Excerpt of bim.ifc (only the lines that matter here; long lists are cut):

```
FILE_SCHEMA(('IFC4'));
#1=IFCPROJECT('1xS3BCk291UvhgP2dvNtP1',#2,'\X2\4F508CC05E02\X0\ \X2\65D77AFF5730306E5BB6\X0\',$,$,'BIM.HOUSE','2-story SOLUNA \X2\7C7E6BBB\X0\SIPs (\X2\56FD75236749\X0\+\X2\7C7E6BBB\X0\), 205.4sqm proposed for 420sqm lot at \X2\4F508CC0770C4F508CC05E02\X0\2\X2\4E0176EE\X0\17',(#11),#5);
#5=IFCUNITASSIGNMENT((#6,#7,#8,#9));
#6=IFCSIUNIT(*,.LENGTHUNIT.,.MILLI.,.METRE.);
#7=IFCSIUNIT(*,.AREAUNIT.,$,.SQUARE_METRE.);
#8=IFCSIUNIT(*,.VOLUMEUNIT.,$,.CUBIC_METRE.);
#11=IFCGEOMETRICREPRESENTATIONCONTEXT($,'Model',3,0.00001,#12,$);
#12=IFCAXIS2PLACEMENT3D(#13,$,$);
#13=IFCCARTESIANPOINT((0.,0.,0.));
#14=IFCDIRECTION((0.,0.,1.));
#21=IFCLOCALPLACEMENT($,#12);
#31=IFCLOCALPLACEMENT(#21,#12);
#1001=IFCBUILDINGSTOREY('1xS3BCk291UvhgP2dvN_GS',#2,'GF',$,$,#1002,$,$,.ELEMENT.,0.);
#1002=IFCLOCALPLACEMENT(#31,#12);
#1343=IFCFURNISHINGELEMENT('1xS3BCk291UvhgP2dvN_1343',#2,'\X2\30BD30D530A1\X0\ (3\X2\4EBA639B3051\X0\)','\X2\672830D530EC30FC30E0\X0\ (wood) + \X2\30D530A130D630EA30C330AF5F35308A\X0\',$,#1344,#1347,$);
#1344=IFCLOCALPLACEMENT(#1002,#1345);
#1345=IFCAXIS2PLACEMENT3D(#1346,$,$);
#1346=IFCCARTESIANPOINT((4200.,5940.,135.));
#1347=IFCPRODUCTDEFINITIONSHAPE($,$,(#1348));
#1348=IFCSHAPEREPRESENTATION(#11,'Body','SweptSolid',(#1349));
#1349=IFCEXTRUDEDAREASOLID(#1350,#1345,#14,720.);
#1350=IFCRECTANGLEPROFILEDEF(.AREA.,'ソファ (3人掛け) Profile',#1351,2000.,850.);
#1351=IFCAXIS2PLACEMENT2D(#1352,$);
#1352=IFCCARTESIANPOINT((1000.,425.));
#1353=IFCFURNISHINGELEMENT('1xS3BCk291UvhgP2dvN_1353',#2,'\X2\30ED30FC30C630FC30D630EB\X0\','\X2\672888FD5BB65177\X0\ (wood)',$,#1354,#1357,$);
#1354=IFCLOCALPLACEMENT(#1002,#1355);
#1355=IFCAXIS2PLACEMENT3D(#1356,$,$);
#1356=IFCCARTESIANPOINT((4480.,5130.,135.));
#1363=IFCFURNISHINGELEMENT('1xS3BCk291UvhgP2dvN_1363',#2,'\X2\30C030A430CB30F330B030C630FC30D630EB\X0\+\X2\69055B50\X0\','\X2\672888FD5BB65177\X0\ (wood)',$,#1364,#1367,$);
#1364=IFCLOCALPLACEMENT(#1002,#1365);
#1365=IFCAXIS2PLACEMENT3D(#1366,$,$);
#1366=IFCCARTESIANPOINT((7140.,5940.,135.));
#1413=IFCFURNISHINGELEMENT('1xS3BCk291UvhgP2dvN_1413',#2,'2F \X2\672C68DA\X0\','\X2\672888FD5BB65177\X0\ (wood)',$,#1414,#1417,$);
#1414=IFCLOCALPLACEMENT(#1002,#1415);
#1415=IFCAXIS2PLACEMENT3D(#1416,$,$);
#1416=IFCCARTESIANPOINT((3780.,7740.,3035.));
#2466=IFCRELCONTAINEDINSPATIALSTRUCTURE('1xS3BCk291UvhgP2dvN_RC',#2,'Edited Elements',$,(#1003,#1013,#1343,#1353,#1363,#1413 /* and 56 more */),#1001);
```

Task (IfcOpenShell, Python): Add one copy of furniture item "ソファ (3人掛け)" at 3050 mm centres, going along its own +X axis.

```python
import ifcopenshell
import ifcopenshell.api.geometry
import ifcopenshell.api.root
import ifcopenshell.util.element
import ifcopenshell.util.placement

model = ifcopenshell.open("bim.ifc")


def reuse_history(source, copy):
    """copy_class also copies each property set's owner history, people and application; keep the originals."""
    for rel in copy.IsDefinedBy:
        if rel.is_a("IfcRelDefinesByProperties") and (history := rel.RelatingPropertyDefinition.OwnerHistory):
            rel.RelatingPropertyDefinition.OwnerHistory = source.OwnerHistory
            ifcopenshell.util.element.remove_deep2(model, history)


source = model.by_guid("1xS3BCk291UvhgP2dvN_1343")
base = ifcopenshell.util.placement.get_local_placement(source.ObjectPlacement)
step = base[:3, 0] * 3050.0

for i in range(1, 2):
    copy = ifcopenshell.api.root.copy_class(model, product=source)
    copy.Representation = ifcopenshell.util.element.copy_deep(
        model, source.Representation, exclude=["IfcGeometricRepresentationContext", "IfcRepresentationMap"]
    )
    reuse_history(source, copy)
    matrix = base.copy()
    matrix[:3, 3] += i * step
    print("added at", matrix[:3, 3].round(3) + 0.0)
    ifcopenshell.api.geometry.edit_object_placement(model, product=copy, matrix=matrix, is_si=False)

model.write("bim_v2.ifc")
```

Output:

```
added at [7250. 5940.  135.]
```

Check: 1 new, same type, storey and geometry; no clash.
